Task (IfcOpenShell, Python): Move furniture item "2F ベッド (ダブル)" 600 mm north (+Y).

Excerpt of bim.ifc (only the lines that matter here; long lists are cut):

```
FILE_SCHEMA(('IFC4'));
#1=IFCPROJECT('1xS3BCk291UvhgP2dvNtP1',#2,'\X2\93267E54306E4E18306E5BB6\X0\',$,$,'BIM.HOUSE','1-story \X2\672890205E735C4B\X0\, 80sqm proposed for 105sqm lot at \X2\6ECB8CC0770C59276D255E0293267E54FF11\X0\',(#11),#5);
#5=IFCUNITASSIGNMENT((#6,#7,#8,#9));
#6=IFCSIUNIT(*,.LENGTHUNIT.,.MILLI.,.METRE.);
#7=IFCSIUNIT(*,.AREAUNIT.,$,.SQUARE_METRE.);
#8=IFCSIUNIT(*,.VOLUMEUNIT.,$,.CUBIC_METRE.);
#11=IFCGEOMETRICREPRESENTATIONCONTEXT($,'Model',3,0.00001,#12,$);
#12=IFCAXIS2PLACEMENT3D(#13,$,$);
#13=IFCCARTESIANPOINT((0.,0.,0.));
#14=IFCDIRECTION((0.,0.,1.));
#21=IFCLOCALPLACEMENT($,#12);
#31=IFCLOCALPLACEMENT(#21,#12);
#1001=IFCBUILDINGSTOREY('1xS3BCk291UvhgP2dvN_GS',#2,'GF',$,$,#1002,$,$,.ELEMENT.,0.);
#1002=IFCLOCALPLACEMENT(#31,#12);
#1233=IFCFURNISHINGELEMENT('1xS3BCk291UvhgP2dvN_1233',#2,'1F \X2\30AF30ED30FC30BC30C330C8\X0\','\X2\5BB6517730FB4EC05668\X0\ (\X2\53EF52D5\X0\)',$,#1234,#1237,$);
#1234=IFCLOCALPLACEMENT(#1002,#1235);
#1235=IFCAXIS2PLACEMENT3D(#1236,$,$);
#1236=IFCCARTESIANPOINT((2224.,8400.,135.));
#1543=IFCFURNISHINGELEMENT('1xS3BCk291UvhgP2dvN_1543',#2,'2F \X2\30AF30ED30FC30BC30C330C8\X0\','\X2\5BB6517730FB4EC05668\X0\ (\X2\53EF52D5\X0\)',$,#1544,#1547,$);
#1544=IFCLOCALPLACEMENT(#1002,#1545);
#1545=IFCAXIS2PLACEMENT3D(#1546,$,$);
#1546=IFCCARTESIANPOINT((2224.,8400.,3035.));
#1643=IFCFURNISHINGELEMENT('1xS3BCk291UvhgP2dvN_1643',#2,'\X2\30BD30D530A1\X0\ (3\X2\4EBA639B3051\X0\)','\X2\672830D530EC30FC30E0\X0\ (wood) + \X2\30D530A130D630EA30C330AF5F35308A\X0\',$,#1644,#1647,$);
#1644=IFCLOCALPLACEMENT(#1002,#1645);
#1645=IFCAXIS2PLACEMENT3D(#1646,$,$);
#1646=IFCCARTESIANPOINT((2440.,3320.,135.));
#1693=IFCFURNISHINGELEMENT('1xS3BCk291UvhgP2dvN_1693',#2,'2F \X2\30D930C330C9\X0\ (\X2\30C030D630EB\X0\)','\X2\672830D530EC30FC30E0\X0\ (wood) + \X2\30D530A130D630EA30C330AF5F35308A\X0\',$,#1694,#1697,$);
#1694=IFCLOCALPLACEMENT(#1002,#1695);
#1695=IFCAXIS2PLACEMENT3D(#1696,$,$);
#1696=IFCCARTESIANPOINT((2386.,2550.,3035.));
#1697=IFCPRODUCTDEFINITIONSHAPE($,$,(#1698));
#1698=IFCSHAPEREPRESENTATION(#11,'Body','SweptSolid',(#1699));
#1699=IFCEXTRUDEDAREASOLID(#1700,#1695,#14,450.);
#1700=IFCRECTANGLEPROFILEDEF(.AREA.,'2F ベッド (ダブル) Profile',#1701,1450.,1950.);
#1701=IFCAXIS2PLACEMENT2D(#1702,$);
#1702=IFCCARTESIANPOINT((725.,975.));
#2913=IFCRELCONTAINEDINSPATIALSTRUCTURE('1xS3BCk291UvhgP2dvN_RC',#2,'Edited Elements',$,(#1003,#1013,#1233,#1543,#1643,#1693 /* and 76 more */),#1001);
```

```python
import ifcopenshell
import ifcopenshell.api.geometry
import ifcopenshell.util.placement
import ifcopenshell.util.unit

model = ifcopenshell.open("bim.ifc")
unit_scale = ifcopenshell.util.unit.calculate_unit_scale(model)

item = model.by_guid("1xS3BCk291UvhgP2dvN_1693")
matrix = ifcopenshell.util.placement.get_local_placement(item.ObjectPlacement)
matrix[1, 3] += 0.6 / unit_scale
ifcopenshell.api.geometry.edit_object_placement(model, product=item, matrix=matrix, is_si=False)

print(ifcopenshell.util.placement.get_local_placement(item.ObjectPlacement).round(3) + 0.0)

model.write("bim-out.ifc")
```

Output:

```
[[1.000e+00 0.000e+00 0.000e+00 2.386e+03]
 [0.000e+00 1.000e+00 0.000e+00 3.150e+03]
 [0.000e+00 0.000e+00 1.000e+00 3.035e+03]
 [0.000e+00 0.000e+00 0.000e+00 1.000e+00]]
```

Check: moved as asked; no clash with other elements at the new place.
